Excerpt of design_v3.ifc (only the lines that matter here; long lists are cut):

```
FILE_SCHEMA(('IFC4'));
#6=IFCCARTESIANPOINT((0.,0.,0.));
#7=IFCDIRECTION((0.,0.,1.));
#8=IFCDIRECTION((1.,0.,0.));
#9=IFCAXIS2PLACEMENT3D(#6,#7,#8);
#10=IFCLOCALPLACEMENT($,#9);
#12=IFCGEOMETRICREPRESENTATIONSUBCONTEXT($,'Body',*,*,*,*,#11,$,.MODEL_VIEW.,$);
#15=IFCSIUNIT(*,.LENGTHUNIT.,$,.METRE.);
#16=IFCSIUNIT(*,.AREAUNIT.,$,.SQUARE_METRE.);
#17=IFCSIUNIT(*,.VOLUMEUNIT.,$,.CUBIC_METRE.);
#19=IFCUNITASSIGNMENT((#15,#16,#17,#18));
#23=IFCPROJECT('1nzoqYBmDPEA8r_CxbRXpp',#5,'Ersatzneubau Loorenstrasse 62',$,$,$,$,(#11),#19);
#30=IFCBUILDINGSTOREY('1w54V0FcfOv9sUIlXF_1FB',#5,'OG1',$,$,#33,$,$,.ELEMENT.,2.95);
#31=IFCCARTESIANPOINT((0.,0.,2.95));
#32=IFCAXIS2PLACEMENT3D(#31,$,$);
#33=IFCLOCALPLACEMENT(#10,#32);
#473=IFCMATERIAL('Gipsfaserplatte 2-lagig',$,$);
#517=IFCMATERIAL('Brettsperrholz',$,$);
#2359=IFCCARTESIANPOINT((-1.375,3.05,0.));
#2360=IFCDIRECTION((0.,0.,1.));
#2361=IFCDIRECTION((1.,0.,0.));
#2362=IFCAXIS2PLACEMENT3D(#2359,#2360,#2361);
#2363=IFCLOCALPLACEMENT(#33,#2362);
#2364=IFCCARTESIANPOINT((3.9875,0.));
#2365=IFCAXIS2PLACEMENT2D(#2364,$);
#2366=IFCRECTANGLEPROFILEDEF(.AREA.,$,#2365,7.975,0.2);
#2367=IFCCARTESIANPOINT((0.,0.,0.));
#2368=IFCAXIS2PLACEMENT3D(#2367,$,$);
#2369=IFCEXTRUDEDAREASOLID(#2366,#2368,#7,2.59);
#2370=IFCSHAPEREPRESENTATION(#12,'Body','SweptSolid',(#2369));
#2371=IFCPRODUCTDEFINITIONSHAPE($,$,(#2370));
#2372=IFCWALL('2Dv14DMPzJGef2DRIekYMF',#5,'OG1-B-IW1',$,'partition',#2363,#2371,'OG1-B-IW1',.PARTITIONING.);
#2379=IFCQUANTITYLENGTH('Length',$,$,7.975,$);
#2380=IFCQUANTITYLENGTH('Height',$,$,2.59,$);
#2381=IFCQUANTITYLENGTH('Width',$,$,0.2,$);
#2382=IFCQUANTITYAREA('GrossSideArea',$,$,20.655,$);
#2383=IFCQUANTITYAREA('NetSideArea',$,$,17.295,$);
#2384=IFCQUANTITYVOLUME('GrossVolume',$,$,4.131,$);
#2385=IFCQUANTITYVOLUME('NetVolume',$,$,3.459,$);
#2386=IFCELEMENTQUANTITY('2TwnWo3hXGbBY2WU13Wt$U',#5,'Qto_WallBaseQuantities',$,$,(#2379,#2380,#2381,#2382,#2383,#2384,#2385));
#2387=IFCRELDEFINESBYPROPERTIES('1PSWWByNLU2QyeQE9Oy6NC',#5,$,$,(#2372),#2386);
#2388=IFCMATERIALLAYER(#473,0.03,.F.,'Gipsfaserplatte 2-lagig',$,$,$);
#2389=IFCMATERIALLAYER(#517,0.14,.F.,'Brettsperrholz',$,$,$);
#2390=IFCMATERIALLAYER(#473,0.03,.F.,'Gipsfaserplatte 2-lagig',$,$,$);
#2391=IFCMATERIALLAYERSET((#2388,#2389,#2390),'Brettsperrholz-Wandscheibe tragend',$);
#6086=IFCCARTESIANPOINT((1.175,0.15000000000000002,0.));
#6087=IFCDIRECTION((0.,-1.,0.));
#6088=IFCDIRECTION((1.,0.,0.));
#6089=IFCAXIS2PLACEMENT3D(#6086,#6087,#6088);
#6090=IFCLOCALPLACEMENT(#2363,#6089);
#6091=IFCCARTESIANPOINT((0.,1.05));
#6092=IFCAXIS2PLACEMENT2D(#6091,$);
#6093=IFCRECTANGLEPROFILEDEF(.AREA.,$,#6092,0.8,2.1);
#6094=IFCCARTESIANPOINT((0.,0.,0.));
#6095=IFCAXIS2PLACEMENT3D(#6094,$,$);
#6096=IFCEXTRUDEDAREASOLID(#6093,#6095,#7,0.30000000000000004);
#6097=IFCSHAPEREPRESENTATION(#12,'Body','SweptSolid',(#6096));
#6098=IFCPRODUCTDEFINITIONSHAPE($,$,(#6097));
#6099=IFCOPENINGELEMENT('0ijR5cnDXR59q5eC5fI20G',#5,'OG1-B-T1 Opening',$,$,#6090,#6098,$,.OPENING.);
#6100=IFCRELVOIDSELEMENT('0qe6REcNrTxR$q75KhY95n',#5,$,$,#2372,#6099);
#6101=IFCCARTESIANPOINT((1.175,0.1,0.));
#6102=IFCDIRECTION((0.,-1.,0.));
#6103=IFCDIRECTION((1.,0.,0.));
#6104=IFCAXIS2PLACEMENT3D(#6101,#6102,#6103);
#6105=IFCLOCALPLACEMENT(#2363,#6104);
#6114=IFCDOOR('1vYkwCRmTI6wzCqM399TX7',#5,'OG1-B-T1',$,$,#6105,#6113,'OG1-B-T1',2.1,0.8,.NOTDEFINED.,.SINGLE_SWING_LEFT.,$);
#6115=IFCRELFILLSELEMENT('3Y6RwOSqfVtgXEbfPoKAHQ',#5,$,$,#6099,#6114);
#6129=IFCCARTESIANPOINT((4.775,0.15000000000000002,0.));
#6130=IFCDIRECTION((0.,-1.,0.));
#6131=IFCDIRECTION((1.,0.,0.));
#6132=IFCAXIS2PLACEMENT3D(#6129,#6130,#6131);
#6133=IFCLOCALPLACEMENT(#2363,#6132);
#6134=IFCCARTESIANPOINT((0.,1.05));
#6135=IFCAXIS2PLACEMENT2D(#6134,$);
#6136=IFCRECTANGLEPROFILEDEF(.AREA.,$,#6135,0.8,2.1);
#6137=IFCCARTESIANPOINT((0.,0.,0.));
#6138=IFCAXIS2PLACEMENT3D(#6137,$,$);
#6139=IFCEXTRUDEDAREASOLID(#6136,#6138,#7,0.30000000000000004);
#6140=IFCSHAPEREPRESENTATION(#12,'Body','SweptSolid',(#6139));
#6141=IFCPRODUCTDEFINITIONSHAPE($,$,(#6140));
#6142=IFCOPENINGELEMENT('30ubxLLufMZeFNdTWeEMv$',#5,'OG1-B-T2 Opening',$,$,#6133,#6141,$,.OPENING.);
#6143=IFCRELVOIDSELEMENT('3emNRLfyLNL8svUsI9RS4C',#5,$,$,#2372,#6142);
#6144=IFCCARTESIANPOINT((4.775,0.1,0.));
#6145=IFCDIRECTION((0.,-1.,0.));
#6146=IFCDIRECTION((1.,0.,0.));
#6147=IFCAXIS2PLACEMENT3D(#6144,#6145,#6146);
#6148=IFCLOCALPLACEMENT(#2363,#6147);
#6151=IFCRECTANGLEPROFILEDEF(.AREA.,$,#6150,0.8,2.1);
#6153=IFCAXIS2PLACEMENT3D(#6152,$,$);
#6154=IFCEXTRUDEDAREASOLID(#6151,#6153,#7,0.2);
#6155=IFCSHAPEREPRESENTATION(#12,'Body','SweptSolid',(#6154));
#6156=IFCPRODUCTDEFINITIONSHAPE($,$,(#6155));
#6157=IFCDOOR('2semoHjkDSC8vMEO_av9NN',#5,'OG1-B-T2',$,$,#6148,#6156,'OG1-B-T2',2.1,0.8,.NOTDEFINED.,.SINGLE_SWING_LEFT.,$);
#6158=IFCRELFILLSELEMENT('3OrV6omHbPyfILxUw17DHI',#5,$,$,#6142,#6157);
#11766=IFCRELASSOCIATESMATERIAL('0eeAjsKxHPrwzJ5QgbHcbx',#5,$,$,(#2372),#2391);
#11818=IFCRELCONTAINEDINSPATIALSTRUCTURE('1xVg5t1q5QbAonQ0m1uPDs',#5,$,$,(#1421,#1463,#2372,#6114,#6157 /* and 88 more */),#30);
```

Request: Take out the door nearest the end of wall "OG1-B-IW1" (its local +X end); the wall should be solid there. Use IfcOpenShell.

```python
import ifcopenshell
import ifcopenshell.api.feature
import ifcopenshell.api.pset
import ifcopenshell.api.root
import ifcopenshell.geom
import ifcopenshell.util.element
import ifcopenshell.util.shape
import ifcopenshell.util.unit

model = ifcopenshell.open("design_v3.ifc")
area_scale = ifcopenshell.util.unit.calculate_unit_scale(model, "AREAUNIT")
volume_scale = ifcopenshell.util.unit.calculate_unit_scale(model, "VOLUMEUNIT")
settings = ifcopenshell.geom.settings()


def volume(element):
    """Net volume in cubic metres, openings subtracted."""
    shape = ifcopenshell.geom.create_shape(settings, element)
    return ifcopenshell.util.shape.get_volume(shape.geometry)


door = model.by_guid("2semoHjkDSC8vMEO_av9NN")
opening = door.FillsVoids[0].RelatingOpeningElement
wall = opening.VoidsElements[0].RelatingBuildingElement
before = volume(wall)

ifcopenshell.api.root.remove_product(model, product=door)
ifcopenshell.api.feature.remove_feature(model, feature=opening)

after = volume(wall)
thickness = 0.2  # wall thickness in metres

# Update the wall's stored quantities.
qto = model.by_id(ifcopenshell.util.element.get_pset(wall, "Qto_WallBaseQuantities", should_inherit=False)["id"])
ifcopenshell.api.pset.edit_qto(model, qto=qto, properties={
    "NetSideArea": after / thickness / area_scale,
    "NetVolume": after / volume_scale,
})

print(f"wall volume {before:.3f} -> {after:.3f} m3")

model.write("design_v3_updated.ifc")
```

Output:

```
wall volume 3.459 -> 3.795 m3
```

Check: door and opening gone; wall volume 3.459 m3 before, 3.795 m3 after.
